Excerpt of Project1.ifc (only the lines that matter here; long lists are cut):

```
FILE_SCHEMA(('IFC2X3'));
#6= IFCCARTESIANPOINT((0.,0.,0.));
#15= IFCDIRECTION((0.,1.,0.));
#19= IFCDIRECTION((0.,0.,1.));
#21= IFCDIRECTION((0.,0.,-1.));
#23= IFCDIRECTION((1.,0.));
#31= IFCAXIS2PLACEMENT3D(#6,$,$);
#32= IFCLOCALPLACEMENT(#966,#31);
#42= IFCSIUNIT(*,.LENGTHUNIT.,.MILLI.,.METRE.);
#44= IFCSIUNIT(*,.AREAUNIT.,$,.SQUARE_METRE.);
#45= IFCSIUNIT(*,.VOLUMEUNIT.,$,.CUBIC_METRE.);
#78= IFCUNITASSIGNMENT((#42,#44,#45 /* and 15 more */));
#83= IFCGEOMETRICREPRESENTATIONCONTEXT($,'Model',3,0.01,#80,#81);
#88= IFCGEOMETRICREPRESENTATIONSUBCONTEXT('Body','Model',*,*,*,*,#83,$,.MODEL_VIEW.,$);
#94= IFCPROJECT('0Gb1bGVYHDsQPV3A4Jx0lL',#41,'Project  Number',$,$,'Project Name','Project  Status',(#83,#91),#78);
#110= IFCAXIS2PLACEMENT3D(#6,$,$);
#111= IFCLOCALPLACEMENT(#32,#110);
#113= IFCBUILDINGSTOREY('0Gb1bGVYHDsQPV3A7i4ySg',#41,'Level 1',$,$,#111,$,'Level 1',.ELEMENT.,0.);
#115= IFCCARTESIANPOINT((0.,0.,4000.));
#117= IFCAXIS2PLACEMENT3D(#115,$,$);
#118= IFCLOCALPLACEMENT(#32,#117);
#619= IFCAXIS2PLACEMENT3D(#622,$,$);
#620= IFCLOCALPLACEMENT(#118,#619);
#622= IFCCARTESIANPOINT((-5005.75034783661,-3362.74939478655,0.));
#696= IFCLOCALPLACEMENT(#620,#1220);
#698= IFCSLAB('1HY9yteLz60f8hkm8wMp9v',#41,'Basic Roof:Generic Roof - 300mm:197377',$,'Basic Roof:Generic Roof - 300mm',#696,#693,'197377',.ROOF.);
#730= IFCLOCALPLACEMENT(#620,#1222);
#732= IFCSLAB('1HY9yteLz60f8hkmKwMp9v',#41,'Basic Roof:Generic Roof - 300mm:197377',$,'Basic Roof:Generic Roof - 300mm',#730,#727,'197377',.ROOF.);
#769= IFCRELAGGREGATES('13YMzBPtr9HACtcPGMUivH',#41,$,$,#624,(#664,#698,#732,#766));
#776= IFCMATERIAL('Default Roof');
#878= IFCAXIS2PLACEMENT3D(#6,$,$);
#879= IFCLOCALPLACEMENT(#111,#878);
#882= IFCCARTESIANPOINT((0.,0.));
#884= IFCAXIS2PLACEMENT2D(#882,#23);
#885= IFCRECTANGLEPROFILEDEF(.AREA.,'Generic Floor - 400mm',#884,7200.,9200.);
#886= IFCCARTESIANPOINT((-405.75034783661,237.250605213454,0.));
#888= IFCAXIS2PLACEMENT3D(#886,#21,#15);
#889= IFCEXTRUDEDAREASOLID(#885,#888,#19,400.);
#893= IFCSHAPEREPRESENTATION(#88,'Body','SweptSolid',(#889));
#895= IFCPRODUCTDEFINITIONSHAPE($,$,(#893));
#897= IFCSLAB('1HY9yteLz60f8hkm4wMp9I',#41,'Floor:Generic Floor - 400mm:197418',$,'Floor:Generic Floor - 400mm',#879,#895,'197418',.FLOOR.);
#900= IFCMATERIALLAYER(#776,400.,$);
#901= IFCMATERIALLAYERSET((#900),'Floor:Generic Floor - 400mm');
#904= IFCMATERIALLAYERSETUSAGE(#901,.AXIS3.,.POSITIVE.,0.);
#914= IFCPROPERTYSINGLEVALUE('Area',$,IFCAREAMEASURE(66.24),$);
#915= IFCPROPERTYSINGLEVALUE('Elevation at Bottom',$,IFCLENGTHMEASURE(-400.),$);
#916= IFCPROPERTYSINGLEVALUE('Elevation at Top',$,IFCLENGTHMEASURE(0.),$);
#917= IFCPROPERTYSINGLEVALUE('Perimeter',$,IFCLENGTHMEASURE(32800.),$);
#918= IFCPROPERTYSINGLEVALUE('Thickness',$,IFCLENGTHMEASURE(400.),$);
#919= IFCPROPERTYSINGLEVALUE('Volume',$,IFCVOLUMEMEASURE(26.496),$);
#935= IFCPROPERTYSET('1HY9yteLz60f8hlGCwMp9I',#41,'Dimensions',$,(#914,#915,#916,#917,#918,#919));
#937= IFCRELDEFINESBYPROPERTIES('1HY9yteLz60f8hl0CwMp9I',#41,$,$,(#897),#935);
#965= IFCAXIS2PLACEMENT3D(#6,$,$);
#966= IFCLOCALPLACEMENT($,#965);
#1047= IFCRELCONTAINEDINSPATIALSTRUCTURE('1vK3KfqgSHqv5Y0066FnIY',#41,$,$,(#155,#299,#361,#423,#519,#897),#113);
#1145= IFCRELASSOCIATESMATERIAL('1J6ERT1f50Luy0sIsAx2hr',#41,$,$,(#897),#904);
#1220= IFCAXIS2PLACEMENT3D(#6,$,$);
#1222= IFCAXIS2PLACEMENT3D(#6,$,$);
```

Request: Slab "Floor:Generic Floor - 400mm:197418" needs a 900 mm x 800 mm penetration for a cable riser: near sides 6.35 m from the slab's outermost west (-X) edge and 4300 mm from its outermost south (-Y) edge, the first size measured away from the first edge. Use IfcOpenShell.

```python
import numpy as np
import ifcopenshell
import ifcopenshell.api.feature
import ifcopenshell.api.geometry
import ifcopenshell.api.pset
import ifcopenshell.api.root
import ifcopenshell.geom
import ifcopenshell.util.element
import ifcopenshell.util.placement
import ifcopenshell.util.representation
import ifcopenshell.util.shape
import ifcopenshell.util.unit

model = ifcopenshell.open("Project1.ifc")
unit_scale = ifcopenshell.util.unit.calculate_unit_scale(model)
area_scale = ifcopenshell.util.unit.calculate_unit_scale(model, "AREAUNIT")
volume_scale = ifcopenshell.util.unit.calculate_unit_scale(model, "VOLUMEUNIT")
settings = ifcopenshell.geom.settings()


def volume(element):
    """Net volume in cubic metres, openings subtracted."""
    shape = ifcopenshell.geom.create_shape(settings, element)
    return ifcopenshell.util.shape.get_volume(shape.geometry)


slab = model.by_guid("1HY9yteLz60f8hkm4wMp9I")
before = volume(slab)

# Extent in the slab's own axes, in metres. The edges named are its -X and -Y sides.
slab_shape = ifcopenshell.geom.create_shape(settings, slab)
vertices = ifcopenshell.util.shape.get_vertices(slab_shape.geometry)
x_min, y_min, bottom = vertices.min(axis=0)
top = vertices[:, 2].max()

opening = ifcopenshell.api.root.create_entity(model, ifc_class="IfcOpeningElement", name="Cable riser opening")
context = ifcopenshell.util.representation.get_context(model, "Model", "Body", "MODEL_VIEW")
width, depth = 0.9, 0.8
outline = [(0.0, 0.0), (width, 0.0), (width, depth), (0.0, depth), (0.0, 0.0)]
# Overshoot both faces by 50 mm so the cut is clean.
shape = ifcopenshell.api.geometry.add_slab_representation(
    model, context=context, depth=top - bottom + 0.1, polyline=outline
)
ifcopenshell.api.geometry.assign_representation(model, product=opening, representation=shape)

matrix = ifcopenshell.util.placement.get_local_placement(slab.ObjectPlacement)
matrix[:, 3] = matrix @ np.append(np.array([x_min + 6.35, y_min + 4.3, bottom - 0.05]) / unit_scale, 1.0)
ifcopenshell.api.geometry.edit_object_placement(model, product=opening, matrix=matrix, is_si=False)
ifcopenshell.api.feature.add_feature(model, feature=opening, element=slab)

after = volume(slab)

# Update the slab's stored quantities.
pset = model.by_id(ifcopenshell.util.element.get_pset(slab, "Dimensions", should_inherit=False)["id"])
ifcopenshell.api.pset.edit_pset(model, pset=pset, properties={
    "Area": model.create_entity("IfcAreaMeasure", after / (top - bottom) / area_scale),
    "Volume": model.create_entity("IfcVolumeMeasure", after / volume_scale),
})

print(f"slab volume {before:.3f} -> {after:.3f} m3")

model.write("Project1_rev.ifc")
```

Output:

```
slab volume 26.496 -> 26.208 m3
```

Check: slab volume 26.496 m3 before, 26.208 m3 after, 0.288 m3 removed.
